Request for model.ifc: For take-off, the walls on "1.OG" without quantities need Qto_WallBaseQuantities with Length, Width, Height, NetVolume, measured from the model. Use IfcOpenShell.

First a look at what the model holds.

```python
import ifcopenshell
import ifcopenshell.util.element
import ifcopenshell.util.unit

model = ifcopenshell.open("model.ifc")
print(model.schema)
for unit_type in ("LENGTHUNIT", "AREAUNIT", "VOLUMEUNIT"):
    print(unit_type, ifcopenshell.util.unit.calculate_unit_scale(model, unit_type))
storey = next(s for s in model.by_type("IfcBuildingStorey") if s.Name == "1.OG")
walls = [e for e in ifcopenshell.util.element.get_decomposition(storey) if e.is_a("IfcWall")]
for e in sorted(walls, key=lambda e: e.id()):
    print(e.id(), e.is_a(), e.Name, list(ifcopenshell.util.element.get_psets(e, qtos_only=True)), sep=" | ")
```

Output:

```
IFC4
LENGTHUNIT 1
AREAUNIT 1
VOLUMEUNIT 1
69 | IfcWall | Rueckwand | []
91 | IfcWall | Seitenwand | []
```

```python
import ifcopenshell
import ifcopenshell.api.pset
import ifcopenshell.geom
import ifcopenshell.util.element
import ifcopenshell.util.shape
import ifcopenshell.util.unit

model = ifcopenshell.open("model.ifc")
unit_scale = ifcopenshell.util.unit.calculate_unit_scale(model)
volume_scale = ifcopenshell.util.unit.calculate_unit_scale(model, "VOLUMEUNIT")
settings = ifcopenshell.geom.settings()

storey = next(s for s in model.by_type("IfcBuildingStorey") if s.Name == "1.OG")
walls = [e for e in ifcopenshell.util.element.get_decomposition(storey) if e.is_a("IfcWall")]

for e in sorted(walls, key=lambda e: e.id()):
    if ifcopenshell.util.element.get_psets(e, qtos_only=True, should_inherit=False):
        continue
    # Geometry comes back in metres, in the element's own axes.
    shape = ifcopenshell.geom.create_shape(settings, e)
    values = {
        "Length": ifcopenshell.util.shape.get_x(shape.geometry) / unit_scale,
        "Width": ifcopenshell.util.shape.get_y(shape.geometry) / unit_scale,
        "Height": ifcopenshell.util.shape.get_z(shape.geometry) / unit_scale,
        "NetVolume": ifcopenshell.util.shape.get_volume(shape.geometry) / volume_scale,
    }
    qto = ifcopenshell.api.pset.add_qto(model, product=e, name="Qto_WallBaseQuantities")
    ifcopenshell.api.pset.edit_qto(model, qto=qto, properties=values)
    print(e.id(), {k: round(v, 3) for k, v in values.items()})

model.write("model-out.ifc")
```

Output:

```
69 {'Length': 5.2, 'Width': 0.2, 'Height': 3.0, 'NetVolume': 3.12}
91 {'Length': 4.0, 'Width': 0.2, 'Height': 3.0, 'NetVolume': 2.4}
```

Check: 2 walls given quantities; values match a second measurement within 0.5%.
